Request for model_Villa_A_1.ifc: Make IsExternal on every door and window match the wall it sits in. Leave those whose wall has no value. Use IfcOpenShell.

First a look at what the model holds.

```python
import ifcopenshell
import ifcopenshell.util.element

model = ifcopenshell.open("model_Villa_A_1.ifc")
print(model.schema)
seen = {}
for e in model.by_type("IfcDoor") + model.by_type("IfcWindow"):
    if not e.FillsVoids:
        continue
    host = e.FillsVoids[0].RelatingOpeningElement.VoidsElements[0].RelatingBuildingElement
    own = ifcopenshell.util.element.get_pset(e, f"Pset_{e.is_a()[3:].removesuffix('StandardCase')}Common", "IsExternal")
    wall = ifcopenshell.util.element.get_pset(host, "Pset_WallCommon", "IsExternal")
    seen[e.is_a(), own, wall] = seen.get((e.is_a(), own, wall), 0) + 1
for (cls, own, wall), count in sorted(seen.items(), key=str):
    print(count, cls, "IsExternal:", own, "| host wall:", wall)
```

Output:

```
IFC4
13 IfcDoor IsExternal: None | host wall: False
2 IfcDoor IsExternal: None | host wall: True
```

```python
import ifcopenshell
import ifcopenshell.api.pset
import ifcopenshell.util.element

model = ifcopenshell.open("model_Villa_A_1.ifc")

count = 0
for ifc_class, pset_name in (("IfcDoor", "Pset_DoorCommon"), ("IfcWindow", "Pset_WindowCommon")):
    for e in model.by_type(ifc_class):
        if not e.FillsVoids:
            continue
        host = e.FillsVoids[0].RelatingOpeningElement.VoidsElements[0].RelatingBuildingElement
        external = ifcopenshell.util.element.get_pset(host, "Pset_WallCommon", "IsExternal")
        if external is None or ifcopenshell.util.element.get_pset(e, pset_name, "IsExternal") == external:
            continue
        pset = ifcopenshell.api.pset.add_pset(model, product=e, name=pset_name)
        ifcopenshell.api.pset.edit_pset(model, pset=pset, properties={"IsExternal": external})
        count += 1

print(count, "updated")

model.write("model_Villa_A_1_updated.ifc")
```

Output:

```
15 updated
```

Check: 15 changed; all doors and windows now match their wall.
